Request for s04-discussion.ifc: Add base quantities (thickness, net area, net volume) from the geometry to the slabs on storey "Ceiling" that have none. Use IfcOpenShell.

First a look at what the model holds.

```python
import ifcopenshell
import ifcopenshell.util.element
import ifcopenshell.util.unit

model = ifcopenshell.open("s04-discussion.ifc")
print(model.schema)
for unit_type in ("LENGTHUNIT", "AREAUNIT", "VOLUMEUNIT"):
    print(unit_type, ifcopenshell.util.unit.calculate_unit_scale(model, unit_type))
storey = next(s for s in model.by_type("IfcBuildingStorey") if s.Name == "Ceiling")
slabs = [e for e in ifcopenshell.util.element.get_decomposition(storey) if e.is_a("IfcSlab")]
for e in sorted(slabs, key=lambda e: e.id()):
    print(e.id(), e.is_a(), e.Name, list(ifcopenshell.util.element.get_psets(e, qtos_only=True)), sep=" | ")
```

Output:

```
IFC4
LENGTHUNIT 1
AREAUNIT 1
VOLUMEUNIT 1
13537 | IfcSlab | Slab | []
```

```python
import ifcopenshell
import ifcopenshell.api.pset
import ifcopenshell.geom
import ifcopenshell.util.element
import ifcopenshell.util.shape
import ifcopenshell.util.unit

model = ifcopenshell.open("s04-discussion.ifc")
unit_scale = ifcopenshell.util.unit.calculate_unit_scale(model)
area_scale = ifcopenshell.util.unit.calculate_unit_scale(model, "AREAUNIT")
volume_scale = ifcopenshell.util.unit.calculate_unit_scale(model, "VOLUMEUNIT")
settings = ifcopenshell.geom.settings()

storey = next(s for s in model.by_type("IfcBuildingStorey") if s.Name == "Ceiling")
slabs = [e for e in ifcopenshell.util.element.get_decomposition(storey) if e.is_a("IfcSlab")]

for e in sorted(slabs, key=lambda e: e.id()):
    if ifcopenshell.util.element.get_psets(e, qtos_only=True, should_inherit=False):
        continue
    # Geometry comes back in metres, in the element's own axes.
    shape = ifcopenshell.geom.create_shape(settings, e)
    values = {
        "Width": ifcopenshell.util.shape.get_z(shape.geometry) / unit_scale,
        "NetArea": ifcopenshell.util.shape.get_footprint_area(shape.geometry) / area_scale,
        "NetVolume": ifcopenshell.util.shape.get_volume(shape.geometry) / volume_scale,
    }
    qto = ifcopenshell.api.pset.add_qto(model, product=e, name="Qto_SlabBaseQuantities")
    ifcopenshell.api.pset.edit_qto(model, qto=qto, properties=values)
    print(e.id(), {k: round(v, 3) for k, v in values.items()})

model.write("s04-discussion_edited.ifc")
```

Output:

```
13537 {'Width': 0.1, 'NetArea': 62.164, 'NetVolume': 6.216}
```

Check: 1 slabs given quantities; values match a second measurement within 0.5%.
